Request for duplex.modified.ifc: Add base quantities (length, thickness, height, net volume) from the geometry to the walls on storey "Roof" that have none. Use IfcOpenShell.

First a look at what the model holds.

```python
import ifcopenshell
import ifcopenshell.util.element
import ifcopenshell.util.unit

model = ifcopenshell.open("duplex.modified.ifc")
print(model.schema)
for unit_type in ("LENGTHUNIT", "AREAUNIT", "VOLUMEUNIT"):
    print(unit_type, ifcopenshell.util.unit.calculate_unit_scale(model, unit_type))
storey = next(s for s in model.by_type("IfcBuildingStorey") if s.Name == "Roof")
walls = [e for e in ifcopenshell.util.element.get_decomposition(storey) if e.is_a("IfcWall")]
for e in sorted(walls, key=lambda e: e.id()):
    print(e.id(), e.is_a(), e.Name, list(ifcopenshell.util.element.get_psets(e, qtos_only=True)), sep=" | ")
```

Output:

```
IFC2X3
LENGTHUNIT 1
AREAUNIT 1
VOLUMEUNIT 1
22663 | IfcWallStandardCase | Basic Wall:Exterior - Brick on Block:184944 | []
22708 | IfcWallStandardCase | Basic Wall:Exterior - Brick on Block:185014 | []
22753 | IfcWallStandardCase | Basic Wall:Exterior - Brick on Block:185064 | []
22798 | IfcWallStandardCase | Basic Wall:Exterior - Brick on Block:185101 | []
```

```python
import ifcopenshell
import ifcopenshell.api.pset
import ifcopenshell.geom
import ifcopenshell.util.element
import ifcopenshell.util.shape
import ifcopenshell.util.unit

model = ifcopenshell.open("duplex.modified.ifc")
unit_scale = ifcopenshell.util.unit.calculate_unit_scale(model)
volume_scale = ifcopenshell.util.unit.calculate_unit_scale(model, "VOLUMEUNIT")
settings = ifcopenshell.geom.settings()

storey = next(s for s in model.by_type("IfcBuildingStorey") if s.Name == "Roof")
walls = [e for e in ifcopenshell.util.element.get_decomposition(storey) if e.is_a("IfcWall")]

for e in sorted(walls, key=lambda e: e.id()):
    if ifcopenshell.util.element.get_psets(e, qtos_only=True, should_inherit=False):
        continue
    # Geometry comes back in metres, in the element's own axes.
    shape = ifcopenshell.geom.create_shape(settings, e)
    values = {
        "Length": ifcopenshell.util.shape.get_x(shape.geometry) / unit_scale,
        "Width": ifcopenshell.util.shape.get_y(shape.geometry) / unit_scale,
        "Height": ifcopenshell.util.shape.get_z(shape.geometry) / unit_scale,
        "NetVolume": ifcopenshell.util.shape.get_volume(shape.geometry) / volume_scale,
    }
    qto = ifcopenshell.api.pset.add_qto(model, product=e, name="BaseQuantities")
    ifcopenshell.api.pset.edit_qto(model, qto=qto, properties=values)
    print(e.id(), {k: round(v, 3) for k, v in values.items()})

model.write("duplex.modified_v2.ifc")
```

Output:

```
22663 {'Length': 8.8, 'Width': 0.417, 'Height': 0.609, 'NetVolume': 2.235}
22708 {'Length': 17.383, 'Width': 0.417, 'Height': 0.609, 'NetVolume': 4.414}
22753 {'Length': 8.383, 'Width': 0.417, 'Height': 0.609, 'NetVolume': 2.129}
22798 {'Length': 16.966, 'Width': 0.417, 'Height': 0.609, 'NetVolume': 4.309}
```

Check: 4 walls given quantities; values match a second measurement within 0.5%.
